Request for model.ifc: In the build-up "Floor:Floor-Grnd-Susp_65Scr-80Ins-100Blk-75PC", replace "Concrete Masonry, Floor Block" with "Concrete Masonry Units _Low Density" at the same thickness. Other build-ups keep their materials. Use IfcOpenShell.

First a look at what the model holds.

```python
import ifcopenshell
import ifcopenshell.util.element

model = ifcopenshell.open("model.ifc")
print(model.schema)
for layer_set in model.by_type("IfcMaterialLayerSet"):
    if layer_set.LayerSetName == "Floor:Floor-Grnd-Susp_65Scr-80Ins-100Blk-75PC":
        for layer in layer_set.MaterialLayers:
            print(layer.id(), layer.Material and layer.Material.Name, layer.LayerThickness, sep=" | ")
        print(len(ifcopenshell.util.element.get_elements_by_material(model, layer_set)), "elements and types use it")
print(sorted(m.Name for m in model.by_type("IfcMaterial") if m.Name)[:60])
```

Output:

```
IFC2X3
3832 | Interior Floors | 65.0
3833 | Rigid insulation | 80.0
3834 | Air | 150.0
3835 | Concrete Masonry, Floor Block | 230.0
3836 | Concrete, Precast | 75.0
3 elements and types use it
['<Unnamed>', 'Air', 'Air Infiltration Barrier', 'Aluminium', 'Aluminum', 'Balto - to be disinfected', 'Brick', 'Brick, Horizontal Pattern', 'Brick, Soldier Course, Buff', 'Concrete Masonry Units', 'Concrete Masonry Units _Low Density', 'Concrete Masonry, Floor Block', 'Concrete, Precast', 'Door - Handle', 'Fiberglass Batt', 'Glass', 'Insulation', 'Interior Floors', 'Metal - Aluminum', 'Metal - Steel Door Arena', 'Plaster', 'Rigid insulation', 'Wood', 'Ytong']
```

```python
import ifcopenshell
import ifcopenshell.api.material

model = ifcopenshell.open("model.ifc")

layer_set = next(s for s in model.by_type("IfcMaterialLayerSet") if s.LayerSetName == "Floor:Floor-Grnd-Susp_65Scr-80Ins-100Blk-75PC")
layer = next(l for l in layer_set.MaterialLayers if l.Material and l.Material.Name == "Concrete Masonry, Floor Block")
material = next(m for m in model.by_type("IfcMaterial") if m.Name == "Concrete Masonry Units _Low Density")

# Point this one layer at the other material; renaming the old one would change it everywhere.
ifcopenshell.api.material.edit_layer(model, layer=layer, attributes={}, material=material)

print([l.Material.Name if l.Material else None for l in layer_set.MaterialLayers])

model.write("model_updated.ifc")
```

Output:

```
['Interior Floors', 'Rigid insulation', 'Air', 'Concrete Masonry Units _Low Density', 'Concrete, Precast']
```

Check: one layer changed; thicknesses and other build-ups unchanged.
